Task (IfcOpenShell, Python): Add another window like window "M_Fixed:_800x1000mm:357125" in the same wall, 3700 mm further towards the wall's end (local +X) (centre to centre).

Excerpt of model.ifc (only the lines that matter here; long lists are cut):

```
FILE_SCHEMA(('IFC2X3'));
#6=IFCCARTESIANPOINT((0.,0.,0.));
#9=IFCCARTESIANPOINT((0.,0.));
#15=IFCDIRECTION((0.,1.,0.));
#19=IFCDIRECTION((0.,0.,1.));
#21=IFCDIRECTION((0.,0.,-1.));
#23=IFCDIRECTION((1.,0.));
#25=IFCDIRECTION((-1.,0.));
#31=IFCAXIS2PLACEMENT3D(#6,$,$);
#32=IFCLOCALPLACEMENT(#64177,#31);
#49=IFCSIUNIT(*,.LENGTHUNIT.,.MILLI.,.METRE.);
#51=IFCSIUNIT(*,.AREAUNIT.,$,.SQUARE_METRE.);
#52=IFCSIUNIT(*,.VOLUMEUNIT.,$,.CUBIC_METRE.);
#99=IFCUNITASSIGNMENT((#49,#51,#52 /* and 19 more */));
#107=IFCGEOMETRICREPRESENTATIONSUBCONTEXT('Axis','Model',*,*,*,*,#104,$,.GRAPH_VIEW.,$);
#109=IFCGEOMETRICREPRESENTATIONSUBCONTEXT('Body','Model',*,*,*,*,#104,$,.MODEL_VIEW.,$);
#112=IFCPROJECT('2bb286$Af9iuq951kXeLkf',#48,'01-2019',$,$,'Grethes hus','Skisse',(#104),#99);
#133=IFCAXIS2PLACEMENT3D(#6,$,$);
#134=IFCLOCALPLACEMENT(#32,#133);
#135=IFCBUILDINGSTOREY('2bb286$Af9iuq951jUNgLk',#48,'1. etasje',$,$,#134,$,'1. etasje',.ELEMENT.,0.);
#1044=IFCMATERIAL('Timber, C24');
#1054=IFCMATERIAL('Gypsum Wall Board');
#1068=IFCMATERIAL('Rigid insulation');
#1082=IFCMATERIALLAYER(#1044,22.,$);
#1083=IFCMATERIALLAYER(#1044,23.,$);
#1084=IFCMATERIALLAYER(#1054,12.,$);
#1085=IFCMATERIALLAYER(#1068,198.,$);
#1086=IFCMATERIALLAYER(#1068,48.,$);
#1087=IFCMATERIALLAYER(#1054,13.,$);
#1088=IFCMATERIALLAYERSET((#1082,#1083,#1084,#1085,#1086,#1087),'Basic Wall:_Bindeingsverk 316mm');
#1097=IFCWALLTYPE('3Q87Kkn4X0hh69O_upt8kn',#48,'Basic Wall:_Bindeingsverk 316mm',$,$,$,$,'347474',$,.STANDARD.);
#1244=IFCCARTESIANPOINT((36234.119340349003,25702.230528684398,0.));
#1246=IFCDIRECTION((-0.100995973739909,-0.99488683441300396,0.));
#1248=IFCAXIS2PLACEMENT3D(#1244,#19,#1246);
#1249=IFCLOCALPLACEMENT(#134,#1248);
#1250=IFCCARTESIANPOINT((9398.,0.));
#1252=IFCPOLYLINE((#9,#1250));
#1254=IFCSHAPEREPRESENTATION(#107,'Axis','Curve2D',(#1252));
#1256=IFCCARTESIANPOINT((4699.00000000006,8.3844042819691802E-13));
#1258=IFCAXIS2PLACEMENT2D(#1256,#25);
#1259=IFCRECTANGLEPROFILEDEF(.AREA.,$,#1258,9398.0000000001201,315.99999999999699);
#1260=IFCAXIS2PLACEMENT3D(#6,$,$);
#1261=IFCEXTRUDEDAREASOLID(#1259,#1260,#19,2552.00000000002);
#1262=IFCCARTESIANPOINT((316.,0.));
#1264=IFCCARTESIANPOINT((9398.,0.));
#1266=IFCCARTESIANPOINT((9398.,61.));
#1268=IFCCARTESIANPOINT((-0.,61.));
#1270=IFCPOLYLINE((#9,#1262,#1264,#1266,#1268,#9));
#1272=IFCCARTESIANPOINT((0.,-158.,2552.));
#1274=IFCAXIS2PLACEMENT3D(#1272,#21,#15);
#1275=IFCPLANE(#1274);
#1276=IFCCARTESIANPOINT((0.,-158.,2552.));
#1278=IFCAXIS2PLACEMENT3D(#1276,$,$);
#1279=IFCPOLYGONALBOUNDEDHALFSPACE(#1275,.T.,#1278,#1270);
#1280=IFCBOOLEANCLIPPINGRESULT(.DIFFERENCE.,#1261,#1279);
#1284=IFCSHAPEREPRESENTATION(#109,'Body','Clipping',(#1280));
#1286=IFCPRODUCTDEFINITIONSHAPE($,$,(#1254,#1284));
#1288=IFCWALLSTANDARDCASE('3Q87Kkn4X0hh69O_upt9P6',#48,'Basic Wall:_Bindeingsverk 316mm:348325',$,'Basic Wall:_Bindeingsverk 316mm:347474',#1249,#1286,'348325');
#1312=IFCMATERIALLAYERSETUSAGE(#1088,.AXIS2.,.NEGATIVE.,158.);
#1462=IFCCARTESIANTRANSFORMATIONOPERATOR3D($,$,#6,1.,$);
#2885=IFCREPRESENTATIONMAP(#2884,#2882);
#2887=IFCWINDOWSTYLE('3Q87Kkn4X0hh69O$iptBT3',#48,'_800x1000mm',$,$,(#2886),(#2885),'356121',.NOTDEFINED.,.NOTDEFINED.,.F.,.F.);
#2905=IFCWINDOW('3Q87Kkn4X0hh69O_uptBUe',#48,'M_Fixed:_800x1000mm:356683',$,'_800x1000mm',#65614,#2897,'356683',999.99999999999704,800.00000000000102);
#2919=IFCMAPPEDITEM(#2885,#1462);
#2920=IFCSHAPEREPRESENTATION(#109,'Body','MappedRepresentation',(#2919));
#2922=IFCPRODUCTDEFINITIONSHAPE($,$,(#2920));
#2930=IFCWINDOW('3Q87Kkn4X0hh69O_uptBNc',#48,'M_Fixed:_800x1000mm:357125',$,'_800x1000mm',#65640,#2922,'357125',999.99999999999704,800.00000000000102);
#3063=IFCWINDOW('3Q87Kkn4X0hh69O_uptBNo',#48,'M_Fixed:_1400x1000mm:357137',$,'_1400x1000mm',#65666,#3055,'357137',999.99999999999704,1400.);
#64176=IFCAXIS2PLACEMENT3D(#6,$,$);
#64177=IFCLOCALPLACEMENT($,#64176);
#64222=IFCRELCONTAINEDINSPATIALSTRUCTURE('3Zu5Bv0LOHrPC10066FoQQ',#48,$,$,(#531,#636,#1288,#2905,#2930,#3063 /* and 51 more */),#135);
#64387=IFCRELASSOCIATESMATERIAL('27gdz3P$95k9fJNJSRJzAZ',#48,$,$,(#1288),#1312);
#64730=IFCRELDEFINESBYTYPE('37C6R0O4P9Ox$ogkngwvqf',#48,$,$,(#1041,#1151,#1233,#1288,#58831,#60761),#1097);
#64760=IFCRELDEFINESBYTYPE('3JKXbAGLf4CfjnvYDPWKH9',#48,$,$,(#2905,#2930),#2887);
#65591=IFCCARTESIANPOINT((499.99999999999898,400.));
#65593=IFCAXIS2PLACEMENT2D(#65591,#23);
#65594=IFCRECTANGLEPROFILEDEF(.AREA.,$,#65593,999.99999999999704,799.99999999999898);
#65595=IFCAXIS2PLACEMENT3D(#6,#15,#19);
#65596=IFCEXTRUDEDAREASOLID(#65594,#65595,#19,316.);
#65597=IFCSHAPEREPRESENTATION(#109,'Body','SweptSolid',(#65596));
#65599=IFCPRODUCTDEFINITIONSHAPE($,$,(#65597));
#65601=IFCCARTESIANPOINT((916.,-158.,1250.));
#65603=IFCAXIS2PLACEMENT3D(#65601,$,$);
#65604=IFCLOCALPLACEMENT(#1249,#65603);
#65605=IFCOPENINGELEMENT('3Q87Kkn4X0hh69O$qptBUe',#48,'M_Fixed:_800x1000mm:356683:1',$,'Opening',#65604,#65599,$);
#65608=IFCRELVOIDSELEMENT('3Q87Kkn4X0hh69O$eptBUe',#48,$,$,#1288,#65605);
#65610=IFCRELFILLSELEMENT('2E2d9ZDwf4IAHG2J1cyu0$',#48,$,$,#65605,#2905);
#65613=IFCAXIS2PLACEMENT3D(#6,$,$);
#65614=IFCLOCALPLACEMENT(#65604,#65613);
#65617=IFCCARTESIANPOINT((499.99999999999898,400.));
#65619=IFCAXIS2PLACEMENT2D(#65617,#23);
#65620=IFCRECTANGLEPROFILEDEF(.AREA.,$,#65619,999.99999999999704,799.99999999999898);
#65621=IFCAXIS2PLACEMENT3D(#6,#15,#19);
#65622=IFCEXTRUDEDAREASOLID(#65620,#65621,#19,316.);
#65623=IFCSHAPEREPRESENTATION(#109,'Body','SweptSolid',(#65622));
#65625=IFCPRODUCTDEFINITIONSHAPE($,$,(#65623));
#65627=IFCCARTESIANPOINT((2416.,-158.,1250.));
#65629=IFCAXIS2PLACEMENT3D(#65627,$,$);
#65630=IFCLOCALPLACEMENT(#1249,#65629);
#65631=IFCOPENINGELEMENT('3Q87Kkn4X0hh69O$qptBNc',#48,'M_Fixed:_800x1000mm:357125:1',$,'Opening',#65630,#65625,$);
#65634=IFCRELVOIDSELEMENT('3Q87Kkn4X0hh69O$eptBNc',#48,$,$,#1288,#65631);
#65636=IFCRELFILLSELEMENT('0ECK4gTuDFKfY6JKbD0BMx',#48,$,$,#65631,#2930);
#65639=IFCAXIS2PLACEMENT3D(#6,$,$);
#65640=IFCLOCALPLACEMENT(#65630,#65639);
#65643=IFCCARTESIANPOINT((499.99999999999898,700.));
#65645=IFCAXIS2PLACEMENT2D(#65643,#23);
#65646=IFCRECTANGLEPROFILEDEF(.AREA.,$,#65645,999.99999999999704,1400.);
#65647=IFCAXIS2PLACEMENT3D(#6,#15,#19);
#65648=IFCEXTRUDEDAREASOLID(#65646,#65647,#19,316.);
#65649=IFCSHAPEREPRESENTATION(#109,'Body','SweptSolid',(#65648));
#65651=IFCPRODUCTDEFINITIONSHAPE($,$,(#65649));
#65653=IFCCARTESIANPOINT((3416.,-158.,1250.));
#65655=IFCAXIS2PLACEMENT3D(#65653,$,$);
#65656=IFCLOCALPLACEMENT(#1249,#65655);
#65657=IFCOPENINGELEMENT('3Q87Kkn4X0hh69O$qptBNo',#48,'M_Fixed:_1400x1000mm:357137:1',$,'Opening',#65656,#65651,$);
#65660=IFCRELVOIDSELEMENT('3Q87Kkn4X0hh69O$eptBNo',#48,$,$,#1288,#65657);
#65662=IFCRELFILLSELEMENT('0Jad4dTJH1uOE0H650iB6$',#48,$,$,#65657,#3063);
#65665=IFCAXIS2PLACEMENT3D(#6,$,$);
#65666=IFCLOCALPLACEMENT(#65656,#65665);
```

```python
import ifcopenshell
import ifcopenshell.api.feature
import ifcopenshell.api.geometry
import ifcopenshell.api.root
import ifcopenshell.geom
import ifcopenshell.util.element
import ifcopenshell.util.placement
import ifcopenshell.util.shape

model = ifcopenshell.open("model.ifc")
settings = ifcopenshell.geom.settings()


def volume(element):
    """Net volume in cubic metres, openings subtracted."""
    shape = ifcopenshell.geom.create_shape(settings, element)
    return ifcopenshell.util.shape.get_volume(shape.geometry)


def reuse_history(source, copy):
    """copy_class also copies each property set's owner history, people and application; keep the originals."""
    for rel in copy.IsDefinedBy:
        if rel.is_a("IfcRelDefinesByProperties") and (history := rel.RelatingPropertyDefinition.OwnerHistory):
            rel.RelatingPropertyDefinition.OwnerHistory = source.OwnerHistory
            ifcopenshell.util.element.remove_deep2(model, history)


window = model.by_guid("3Q87Kkn4X0hh69O_uptBNc")
opening = window.FillsVoids[0].RelatingOpeningElement
wall = opening.VoidsElements[0].RelatingBuildingElement
before = volume(wall)
shift = ifcopenshell.util.placement.get_local_placement(wall.ObjectPlacement)[:3, 0] * 3700.0

# copy_class copies the void relationship, type, container and properties, but no geometry.
new_opening = ifcopenshell.api.root.copy_class(model, product=opening)
new_opening.Representation = ifcopenshell.util.element.copy_deep(
    model, opening.Representation, exclude=["IfcGeometricRepresentationContext", "IfcRepresentationMap"]
)
new_opening.Name = "M_Fixed:_800x1000mm"
new_window = ifcopenshell.api.root.copy_class(model, product=window)
new_window.Representation = ifcopenshell.util.element.copy_deep(
    model, window.Representation, exclude=["IfcGeometricRepresentationContext", "IfcRepresentationMap"]
)
new_window.Name = "M_Fixed:_800x1000mm"
new_window.Tag = None
reuse_history(window, new_window)
fills = ifcopenshell.api.feature.add_filling(model, opening=new_opening, element=new_window)
fills.OwnerHistory = new_window.OwnerHistory  # required in IFC2X3

for old, new in ((opening, new_opening), (window, new_window)):
    matrix = ifcopenshell.util.placement.get_local_placement(old.ObjectPlacement)
    matrix[:3, 3] += shift
    ifcopenshell.api.geometry.edit_object_placement(model, product=new, matrix=matrix, is_si=False)

after = volume(wall)

print(f"wall volume {before:.3f} -> {after:.3f} m3")

model.write("model-out.ifc")
```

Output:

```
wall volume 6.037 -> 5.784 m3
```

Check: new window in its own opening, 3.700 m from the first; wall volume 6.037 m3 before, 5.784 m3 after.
